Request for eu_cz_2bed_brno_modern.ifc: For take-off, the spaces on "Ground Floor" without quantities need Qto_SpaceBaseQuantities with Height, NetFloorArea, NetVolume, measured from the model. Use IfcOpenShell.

First a look at what the model holds.

```python
import ifcopenshell
import ifcopenshell.util.element
import ifcopenshell.util.unit

model = ifcopenshell.open("eu_cz_2bed_brno_modern.ifc")
print(model.schema)
for unit_type in ("LENGTHUNIT", "AREAUNIT", "VOLUMEUNIT"):
    print(unit_type, ifcopenshell.util.unit.calculate_unit_scale(model, unit_type))
storey = next(s for s in model.by_type("IfcBuildingStorey") if s.Name == "Ground Floor")
spaces = [e for e in ifcopenshell.util.element.get_decomposition(storey) if e.is_a("IfcSpace")]
for e in sorted(spaces, key=lambda e: e.id()):
    print(e.id(), e.is_a(), e.Name, list(ifcopenshell.util.element.get_psets(e, qtos_only=True)), sep=" | ")
```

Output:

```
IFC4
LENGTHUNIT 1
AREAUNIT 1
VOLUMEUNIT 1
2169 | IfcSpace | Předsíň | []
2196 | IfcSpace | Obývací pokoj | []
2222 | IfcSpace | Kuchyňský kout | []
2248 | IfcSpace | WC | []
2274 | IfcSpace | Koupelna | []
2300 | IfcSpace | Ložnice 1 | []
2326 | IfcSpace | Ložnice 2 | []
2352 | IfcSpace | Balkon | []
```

```python
import ifcopenshell
import ifcopenshell.api.pset
import ifcopenshell.geom
import ifcopenshell.util.element
import ifcopenshell.util.shape
import ifcopenshell.util.unit

model = ifcopenshell.open("eu_cz_2bed_brno_modern.ifc")
unit_scale = ifcopenshell.util.unit.calculate_unit_scale(model)
area_scale = ifcopenshell.util.unit.calculate_unit_scale(model, "AREAUNIT")
volume_scale = ifcopenshell.util.unit.calculate_unit_scale(model, "VOLUMEUNIT")
settings = ifcopenshell.geom.settings()

storey = next(s for s in model.by_type("IfcBuildingStorey") if s.Name == "Ground Floor")
spaces = [e for e in ifcopenshell.util.element.get_decomposition(storey) if e.is_a("IfcSpace")]

for e in sorted(spaces, key=lambda e: e.id()):
    if ifcopenshell.util.element.get_psets(e, qtos_only=True, should_inherit=False):
        continue
    # Geometry comes back in metres, in the element's own axes.
    shape = ifcopenshell.geom.create_shape(settings, e)
    values = {
        "Height": ifcopenshell.util.shape.get_z(shape.geometry) / unit_scale,
        "NetFloorArea": ifcopenshell.util.shape.get_footprint_area(shape.geometry) / area_scale,
        "NetVolume": ifcopenshell.util.shape.get_volume(shape.geometry) / volume_scale,
    }
    qto = ifcopenshell.api.pset.add_qto(model, product=e, name="Qto_SpaceBaseQuantities")
    ifcopenshell.api.pset.edit_qto(model, qto=qto, properties=values)
    print(e.id(), {k: round(v, 3) for k, v in values.items()})

model.write("eu_cz_2bed_brno_modern_edited.ifc")
```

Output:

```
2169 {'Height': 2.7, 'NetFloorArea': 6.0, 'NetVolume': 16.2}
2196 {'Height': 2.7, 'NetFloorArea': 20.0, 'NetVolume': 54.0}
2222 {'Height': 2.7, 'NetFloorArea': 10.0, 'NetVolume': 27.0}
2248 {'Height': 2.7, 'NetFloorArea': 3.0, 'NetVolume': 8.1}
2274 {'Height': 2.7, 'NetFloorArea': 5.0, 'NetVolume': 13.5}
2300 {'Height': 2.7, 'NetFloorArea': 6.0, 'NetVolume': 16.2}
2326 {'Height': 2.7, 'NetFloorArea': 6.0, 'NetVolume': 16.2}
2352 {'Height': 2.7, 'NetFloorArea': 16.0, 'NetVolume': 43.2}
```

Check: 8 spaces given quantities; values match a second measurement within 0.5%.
